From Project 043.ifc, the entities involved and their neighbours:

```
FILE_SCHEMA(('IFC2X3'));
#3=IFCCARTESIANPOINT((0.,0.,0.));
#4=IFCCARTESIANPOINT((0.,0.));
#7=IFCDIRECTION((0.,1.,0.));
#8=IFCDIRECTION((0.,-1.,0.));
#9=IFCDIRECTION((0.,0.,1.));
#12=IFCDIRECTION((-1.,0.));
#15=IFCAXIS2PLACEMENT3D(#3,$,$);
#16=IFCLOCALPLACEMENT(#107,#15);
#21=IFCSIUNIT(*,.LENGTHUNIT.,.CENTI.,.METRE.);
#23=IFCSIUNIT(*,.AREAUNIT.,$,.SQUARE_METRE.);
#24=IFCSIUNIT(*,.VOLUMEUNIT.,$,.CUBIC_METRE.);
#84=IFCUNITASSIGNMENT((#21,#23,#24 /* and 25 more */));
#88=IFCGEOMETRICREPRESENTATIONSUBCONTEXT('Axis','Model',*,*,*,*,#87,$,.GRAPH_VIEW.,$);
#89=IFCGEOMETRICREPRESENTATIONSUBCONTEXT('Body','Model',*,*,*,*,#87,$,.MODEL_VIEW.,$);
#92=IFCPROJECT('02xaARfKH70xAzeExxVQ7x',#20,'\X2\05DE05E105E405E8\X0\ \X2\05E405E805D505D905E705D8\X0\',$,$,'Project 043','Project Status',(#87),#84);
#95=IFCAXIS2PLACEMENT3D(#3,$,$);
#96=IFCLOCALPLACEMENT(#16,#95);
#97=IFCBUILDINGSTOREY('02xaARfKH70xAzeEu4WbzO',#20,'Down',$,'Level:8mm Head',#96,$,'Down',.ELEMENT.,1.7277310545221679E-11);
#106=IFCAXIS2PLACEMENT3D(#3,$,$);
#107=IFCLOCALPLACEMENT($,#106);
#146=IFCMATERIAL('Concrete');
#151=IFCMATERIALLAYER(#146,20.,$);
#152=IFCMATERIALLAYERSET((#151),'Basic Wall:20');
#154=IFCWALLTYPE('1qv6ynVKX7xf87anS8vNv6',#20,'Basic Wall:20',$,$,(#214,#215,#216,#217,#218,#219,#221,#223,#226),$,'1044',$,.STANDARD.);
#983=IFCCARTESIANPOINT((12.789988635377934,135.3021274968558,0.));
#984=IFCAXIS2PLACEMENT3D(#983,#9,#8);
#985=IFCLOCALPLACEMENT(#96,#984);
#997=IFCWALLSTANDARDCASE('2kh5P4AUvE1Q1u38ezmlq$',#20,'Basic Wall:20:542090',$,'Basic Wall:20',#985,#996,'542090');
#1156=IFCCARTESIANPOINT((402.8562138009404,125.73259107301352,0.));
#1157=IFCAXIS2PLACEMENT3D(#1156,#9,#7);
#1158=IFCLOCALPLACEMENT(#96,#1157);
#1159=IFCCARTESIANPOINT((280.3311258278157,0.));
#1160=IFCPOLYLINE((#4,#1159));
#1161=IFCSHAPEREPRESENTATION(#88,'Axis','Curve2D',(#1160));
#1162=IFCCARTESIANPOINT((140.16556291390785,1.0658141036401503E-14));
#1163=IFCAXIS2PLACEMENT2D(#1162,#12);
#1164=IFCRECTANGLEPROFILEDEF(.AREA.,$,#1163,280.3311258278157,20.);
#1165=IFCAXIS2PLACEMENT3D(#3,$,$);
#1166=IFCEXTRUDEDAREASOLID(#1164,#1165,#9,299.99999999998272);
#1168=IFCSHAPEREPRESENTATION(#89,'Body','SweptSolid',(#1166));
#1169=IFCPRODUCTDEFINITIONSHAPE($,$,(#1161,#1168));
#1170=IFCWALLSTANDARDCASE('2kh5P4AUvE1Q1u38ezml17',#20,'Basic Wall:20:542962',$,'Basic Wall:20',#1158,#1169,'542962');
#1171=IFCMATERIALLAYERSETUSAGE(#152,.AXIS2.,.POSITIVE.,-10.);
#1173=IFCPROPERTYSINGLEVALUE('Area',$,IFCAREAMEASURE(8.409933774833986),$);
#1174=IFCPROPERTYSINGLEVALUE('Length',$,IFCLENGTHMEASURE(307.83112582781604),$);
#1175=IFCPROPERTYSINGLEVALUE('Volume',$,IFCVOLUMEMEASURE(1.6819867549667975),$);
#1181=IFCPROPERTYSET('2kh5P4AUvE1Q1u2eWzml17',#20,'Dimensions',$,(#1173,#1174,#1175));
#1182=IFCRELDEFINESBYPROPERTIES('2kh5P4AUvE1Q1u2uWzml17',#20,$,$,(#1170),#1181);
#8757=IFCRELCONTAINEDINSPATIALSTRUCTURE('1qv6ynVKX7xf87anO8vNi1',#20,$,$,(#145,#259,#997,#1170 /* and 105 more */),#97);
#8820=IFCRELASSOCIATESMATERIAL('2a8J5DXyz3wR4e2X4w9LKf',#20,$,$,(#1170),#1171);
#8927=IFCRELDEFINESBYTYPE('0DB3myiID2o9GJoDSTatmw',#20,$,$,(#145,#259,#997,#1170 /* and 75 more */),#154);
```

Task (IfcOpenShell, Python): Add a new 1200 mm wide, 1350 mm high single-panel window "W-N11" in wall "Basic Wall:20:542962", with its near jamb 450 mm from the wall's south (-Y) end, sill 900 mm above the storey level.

```python
import numpy as np
import ifcopenshell
import ifcopenshell.api.feature
import ifcopenshell.api.geometry
import ifcopenshell.api.pset
import ifcopenshell.api.root
import ifcopenshell.api.spatial
import ifcopenshell.api.type
import ifcopenshell.geom
import ifcopenshell.util.element
import ifcopenshell.util.placement
import ifcopenshell.util.representation
import ifcopenshell.util.shape
import ifcopenshell.util.unit

model = ifcopenshell.open("Project 043.ifc")
unit_scale = ifcopenshell.util.unit.calculate_unit_scale(model)
area_scale = ifcopenshell.util.unit.calculate_unit_scale(model, "AREAUNIT")
volume_scale = ifcopenshell.util.unit.calculate_unit_scale(model, "VOLUMEUNIT")
settings = ifcopenshell.geom.settings()


def volume(element):
    """Net volume in cubic metres, openings subtracted."""
    shape = ifcopenshell.geom.create_shape(settings, element)
    return ifcopenshell.util.shape.get_volume(shape.geometry)


wall = model.by_guid("2kh5P4AUvE1Q1u38ezml17")
storey = ifcopenshell.util.element.get_container(wall, ifc_class="IfcBuildingStorey")
context = ifcopenshell.util.representation.get_context(model, "Model", "Body", "MODEL_VIEW")
before = volume(wall)

width, height, from_end, sill = 1.2, 1.35, 0.45, 0.9  # metres

# The wall runs along its own X axis, and the end named is its -X end.
wall_shape = ifcopenshell.geom.create_shape(settings, wall)
x, y, z = ifcopenshell.util.shape.get_vertices(wall_shape.geometry).T
start = x.min() + from_end
face, thickness = float(y.min()), float(y.max() - y.min())
wall_matrix = ifcopenshell.util.placement.get_local_placement(wall.ObjectPlacement)
level = ifcopenshell.util.placement.get_local_placement(storey.ObjectPlacement)[2, 3]


def in_wall(x, y):
    """Placement at x, y metres in the wall's axes, at sill height."""
    matrix = wall_matrix.copy()
    matrix[:, 3] = wall_matrix @ np.array([x / unit_scale, y / unit_scale, 0.0, 1.0])
    matrix[2, 3] = level + sill / unit_scale
    return matrix


# Opening: a box that overshoots both wall faces by 50 mm.
opening = ifcopenshell.api.root.create_entity(model, ifc_class="IfcOpeningElement")
box = ifcopenshell.api.geometry.add_wall_representation(
    model, context=context, length=width, height=height, thickness=thickness + 0.1
)
ifcopenshell.api.geometry.assign_representation(model, product=opening, representation=box)
ifcopenshell.api.geometry.edit_object_placement(model, product=opening, matrix=in_wall(start, face - 0.05), is_si=False)
ifcopenshell.api.feature.add_feature(model, feature=opening, element=wall)

window = ifcopenshell.api.root.create_entity(model, ifc_class="IfcWindow", name="W-N11")
window.OverallWidth, window.OverallHeight = width / unit_scale, height / unit_scale
body = ifcopenshell.api.geometry.add_window_representation(
    model,
    context=context,
    overall_width=window.OverallWidth,
    overall_height=window.OverallHeight,
    partition_type="SINGLE_PANEL",
)
ifcopenshell.api.geometry.assign_representation(model, product=window, representation=body)
ifcopenshell.api.spatial.assign_container(model, products=[window], relating_structure=storey)
fills = ifcopenshell.api.feature.add_filling(model, opening=opening, element=window)
fills.OwnerHistory = window.OwnerHistory  # required in IFC2X3

# IFC2X3 keeps the operation on the window style.
style = ifcopenshell.api.root.create_entity(model, ifc_class="IfcWindowStyle", name="W-N11")
style.OperationType, style.ConstructionType = "SINGLE_PANEL", "NOTDEFINED"
style.ParameterTakesPrecedence = style.Sizeable = False
ifcopenshell.api.type.assign_type(model, related_objects=[window], relating_type=style)

# Centre the window in the wall's thickness.
ifcopenshell.api.geometry.edit_object_placement(model, product=window, matrix=in_wall(start, face), is_si=False)
window_shape = ifcopenshell.geom.create_shape(settings, window)
depth = ifcopenshell.util.shape.get_vertices(window_shape.geometry)[:, 1]
offset = face + thickness / 2 - (depth.min() + depth.max()) / 2
ifcopenshell.api.geometry.edit_object_placement(model, product=window, matrix=in_wall(start, offset), is_si=False)

after = volume(wall)

# Update the wall's stored quantities.
pset = model.by_id(ifcopenshell.util.element.get_pset(wall, "Dimensions", should_inherit=False)["id"])
ifcopenshell.api.pset.edit_pset(model, pset=pset, properties={
    "Area": model.create_entity("IfcAreaMeasure", after / thickness / area_scale),
    "Volume": model.create_entity("IfcVolumeMeasure", after / volume_scale),
})

print(f"wall volume {before:.3f} -> {after:.3f} m3")

model.write("Project 043_v2.ifc")
```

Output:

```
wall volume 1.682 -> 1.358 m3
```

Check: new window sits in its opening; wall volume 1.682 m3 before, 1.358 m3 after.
